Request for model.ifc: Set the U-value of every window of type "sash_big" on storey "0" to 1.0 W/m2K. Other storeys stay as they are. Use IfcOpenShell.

First a look at what the model holds.

```python
import ifcopenshell
import ifcopenshell.util.element

model = ifcopenshell.open("model.ifc")
print(model.schema)
storey = next(s for s in model.by_type("IfcBuildingStorey") if s.Name == "0")
windows = [e for e in ifcopenshell.util.element.get_decomposition(storey) if e.is_a("IfcWindow")]
seen = {}
for e in windows:
    element_type = ifcopenshell.util.element.get_type(e)
    key = (element_type.Name if element_type != e and element_type else None, ifcopenshell.util.element.get_pset(e, "Pset_WindowCommon", "ThermalTransmittance"))
    seen[key] = seen.get(key, 0) + 1
for (name, value), count in sorted(seen.items(), key=str):
    print(count, "x", name, "|", value)
```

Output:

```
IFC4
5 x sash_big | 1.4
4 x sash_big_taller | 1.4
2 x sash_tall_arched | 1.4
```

```python
import ifcopenshell
import ifcopenshell.api.pset
import ifcopenshell.util.element

model = ifcopenshell.open("model.ifc")

storey = next(s for s in model.by_type("IfcBuildingStorey") if s.Name == "0")
windows = [e for e in ifcopenshell.util.element.get_decomposition(storey) if e.is_a("IfcWindow")]

count = 0
for e in windows:
    element_type = ifcopenshell.util.element.get_type(e)
    if element_type in (None, e) or element_type.Name != "sash_big":
        continue
    # add_pset returns the element's existing set when there is one.
    pset = ifcopenshell.api.pset.add_pset(model, product=e, name="Pset_WindowCommon")
    ifcopenshell.api.pset.edit_pset(model, pset=pset, properties={"ThermalTransmittance": 1.0})
    count += 1

print(count, "windows updated")

model.write("model_updated.ifc")
```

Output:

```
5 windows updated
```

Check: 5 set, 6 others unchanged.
